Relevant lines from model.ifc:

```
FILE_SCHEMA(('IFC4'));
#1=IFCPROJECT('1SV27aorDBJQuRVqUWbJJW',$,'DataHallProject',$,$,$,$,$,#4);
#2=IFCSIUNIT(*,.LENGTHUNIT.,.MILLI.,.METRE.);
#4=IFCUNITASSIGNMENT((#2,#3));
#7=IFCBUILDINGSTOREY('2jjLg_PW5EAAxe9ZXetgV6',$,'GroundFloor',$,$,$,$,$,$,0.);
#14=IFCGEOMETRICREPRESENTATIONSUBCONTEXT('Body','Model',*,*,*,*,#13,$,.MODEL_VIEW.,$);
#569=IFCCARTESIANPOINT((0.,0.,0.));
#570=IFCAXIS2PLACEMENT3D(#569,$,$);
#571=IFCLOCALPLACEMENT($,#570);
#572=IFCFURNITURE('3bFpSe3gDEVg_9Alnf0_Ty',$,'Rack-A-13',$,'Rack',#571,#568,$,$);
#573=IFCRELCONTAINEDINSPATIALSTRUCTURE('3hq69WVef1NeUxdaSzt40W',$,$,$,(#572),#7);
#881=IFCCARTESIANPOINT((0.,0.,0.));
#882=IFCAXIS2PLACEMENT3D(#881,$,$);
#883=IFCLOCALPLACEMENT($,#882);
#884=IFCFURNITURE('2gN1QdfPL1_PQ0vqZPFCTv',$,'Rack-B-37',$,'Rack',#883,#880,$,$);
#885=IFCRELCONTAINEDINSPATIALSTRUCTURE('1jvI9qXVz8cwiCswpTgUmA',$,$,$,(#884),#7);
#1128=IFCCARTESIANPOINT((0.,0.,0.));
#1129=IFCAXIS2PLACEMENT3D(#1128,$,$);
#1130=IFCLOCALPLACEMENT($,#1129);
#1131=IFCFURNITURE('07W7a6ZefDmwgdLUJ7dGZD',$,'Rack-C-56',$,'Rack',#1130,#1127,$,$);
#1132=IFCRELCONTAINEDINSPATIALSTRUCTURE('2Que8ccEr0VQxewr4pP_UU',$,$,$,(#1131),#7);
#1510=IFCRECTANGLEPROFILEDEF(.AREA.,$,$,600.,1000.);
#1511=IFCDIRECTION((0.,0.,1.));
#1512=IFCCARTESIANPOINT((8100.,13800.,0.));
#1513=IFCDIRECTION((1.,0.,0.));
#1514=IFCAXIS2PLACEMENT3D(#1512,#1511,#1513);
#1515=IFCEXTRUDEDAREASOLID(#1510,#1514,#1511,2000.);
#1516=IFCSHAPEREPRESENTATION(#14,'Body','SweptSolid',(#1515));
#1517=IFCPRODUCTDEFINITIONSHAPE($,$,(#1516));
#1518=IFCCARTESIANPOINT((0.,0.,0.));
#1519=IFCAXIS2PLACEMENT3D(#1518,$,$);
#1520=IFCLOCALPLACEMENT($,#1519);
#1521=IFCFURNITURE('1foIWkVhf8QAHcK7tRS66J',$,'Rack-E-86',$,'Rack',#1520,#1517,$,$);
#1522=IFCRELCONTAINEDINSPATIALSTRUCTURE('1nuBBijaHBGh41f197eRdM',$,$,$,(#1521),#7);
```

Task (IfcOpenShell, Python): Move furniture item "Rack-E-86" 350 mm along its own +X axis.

```python
import ifcopenshell
import ifcopenshell.api.geometry
import ifcopenshell.util.placement
import ifcopenshell.util.unit

model = ifcopenshell.open("model.ifc")
unit_scale = ifcopenshell.util.unit.calculate_unit_scale(model)

item = model.by_id(1521)
matrix = ifcopenshell.util.placement.get_local_placement(item.ObjectPlacement)
matrix[:3, 3] += matrix[:3, 0] * 0.35 / unit_scale
ifcopenshell.api.geometry.edit_object_placement(model, product=item, matrix=matrix, is_si=False)

print(ifcopenshell.util.placement.get_local_placement(item.ObjectPlacement).round(3) + 0.0)

model.write("model_v2.ifc")
```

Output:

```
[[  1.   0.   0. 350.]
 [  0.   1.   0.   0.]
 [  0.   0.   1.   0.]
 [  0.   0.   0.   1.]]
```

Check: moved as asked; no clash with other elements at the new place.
